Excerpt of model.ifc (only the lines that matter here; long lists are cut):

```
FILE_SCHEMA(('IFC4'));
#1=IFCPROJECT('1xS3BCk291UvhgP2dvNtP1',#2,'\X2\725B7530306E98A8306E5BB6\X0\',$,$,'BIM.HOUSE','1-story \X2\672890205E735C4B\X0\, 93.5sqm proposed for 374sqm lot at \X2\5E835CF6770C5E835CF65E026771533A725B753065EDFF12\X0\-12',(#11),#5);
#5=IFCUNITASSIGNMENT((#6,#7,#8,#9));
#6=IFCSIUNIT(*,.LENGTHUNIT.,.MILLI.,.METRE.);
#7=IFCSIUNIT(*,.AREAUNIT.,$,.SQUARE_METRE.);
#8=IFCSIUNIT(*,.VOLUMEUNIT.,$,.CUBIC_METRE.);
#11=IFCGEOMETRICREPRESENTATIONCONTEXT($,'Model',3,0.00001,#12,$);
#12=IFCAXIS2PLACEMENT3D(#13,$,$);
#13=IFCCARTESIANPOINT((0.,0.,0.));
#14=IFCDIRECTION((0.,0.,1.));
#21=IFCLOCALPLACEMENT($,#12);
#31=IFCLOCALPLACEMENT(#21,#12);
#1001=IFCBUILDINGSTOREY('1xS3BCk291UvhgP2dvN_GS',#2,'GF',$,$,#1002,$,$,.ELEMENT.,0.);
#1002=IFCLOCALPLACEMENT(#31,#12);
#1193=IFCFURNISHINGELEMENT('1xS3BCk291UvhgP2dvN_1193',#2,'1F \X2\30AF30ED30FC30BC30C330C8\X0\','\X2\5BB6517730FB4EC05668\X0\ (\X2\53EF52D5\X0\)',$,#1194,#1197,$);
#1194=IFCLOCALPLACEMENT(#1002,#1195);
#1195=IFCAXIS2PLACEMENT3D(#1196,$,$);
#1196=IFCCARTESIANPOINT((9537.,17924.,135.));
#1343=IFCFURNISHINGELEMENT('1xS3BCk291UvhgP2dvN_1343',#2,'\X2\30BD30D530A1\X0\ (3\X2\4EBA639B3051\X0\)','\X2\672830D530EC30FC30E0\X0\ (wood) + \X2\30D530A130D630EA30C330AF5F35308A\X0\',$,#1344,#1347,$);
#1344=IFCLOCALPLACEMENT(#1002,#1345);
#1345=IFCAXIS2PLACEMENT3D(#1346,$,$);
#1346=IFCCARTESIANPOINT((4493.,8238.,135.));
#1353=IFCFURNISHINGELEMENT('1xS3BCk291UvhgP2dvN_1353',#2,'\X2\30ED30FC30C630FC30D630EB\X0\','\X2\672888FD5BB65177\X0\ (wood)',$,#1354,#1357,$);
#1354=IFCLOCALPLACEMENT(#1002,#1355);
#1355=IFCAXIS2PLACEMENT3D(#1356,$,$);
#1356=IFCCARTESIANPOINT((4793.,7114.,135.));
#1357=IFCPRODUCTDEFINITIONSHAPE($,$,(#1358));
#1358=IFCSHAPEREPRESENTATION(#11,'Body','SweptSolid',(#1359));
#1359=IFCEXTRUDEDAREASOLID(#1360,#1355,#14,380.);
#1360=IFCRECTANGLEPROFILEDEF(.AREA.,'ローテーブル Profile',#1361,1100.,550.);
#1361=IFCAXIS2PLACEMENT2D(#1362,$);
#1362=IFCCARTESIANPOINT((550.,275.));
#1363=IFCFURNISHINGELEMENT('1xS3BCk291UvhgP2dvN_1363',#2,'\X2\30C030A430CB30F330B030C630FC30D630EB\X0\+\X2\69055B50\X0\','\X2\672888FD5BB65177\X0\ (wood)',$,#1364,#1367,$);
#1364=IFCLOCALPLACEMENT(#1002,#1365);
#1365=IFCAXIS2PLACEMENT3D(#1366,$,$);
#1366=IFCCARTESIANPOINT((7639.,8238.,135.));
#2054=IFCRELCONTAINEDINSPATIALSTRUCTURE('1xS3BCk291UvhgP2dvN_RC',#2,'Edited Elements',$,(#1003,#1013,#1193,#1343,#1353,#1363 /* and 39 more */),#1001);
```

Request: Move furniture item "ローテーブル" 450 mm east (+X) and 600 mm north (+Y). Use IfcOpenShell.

```python
import ifcopenshell
import ifcopenshell.api.geometry
import ifcopenshell.util.placement

model = ifcopenshell.open("model.ifc")

item = model.by_id(1353)
matrix = ifcopenshell.util.placement.get_local_placement(item.ObjectPlacement)
matrix[0, 3] += 450.0
matrix[1, 3] += 600.0
ifcopenshell.api.geometry.edit_object_placement(model, product=item, matrix=matrix, is_si=False)

print(ifcopenshell.util.placement.get_local_placement(item.ObjectPlacement).round(3) + 0.0)

model.write("model_rev.ifc")
```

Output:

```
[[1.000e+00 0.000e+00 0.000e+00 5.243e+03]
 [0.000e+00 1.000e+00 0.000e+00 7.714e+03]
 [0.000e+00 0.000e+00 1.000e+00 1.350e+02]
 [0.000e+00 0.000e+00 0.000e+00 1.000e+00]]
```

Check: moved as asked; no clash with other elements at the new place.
